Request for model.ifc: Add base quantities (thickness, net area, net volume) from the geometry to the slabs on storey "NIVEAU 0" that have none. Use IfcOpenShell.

First a look at what the model holds.

```python
import ifcopenshell
import ifcopenshell.util.element
import ifcopenshell.util.unit

model = ifcopenshell.open("model.ifc")
print(model.schema)
for unit_type in ("LENGTHUNIT", "AREAUNIT", "VOLUMEUNIT"):
    print(unit_type, ifcopenshell.util.unit.calculate_unit_scale(model, unit_type))
storey = next(s for s in model.by_type("IfcBuildingStorey") if s.Name == "NIVEAU 0")
slabs = [e for e in ifcopenshell.util.element.get_decomposition(storey) if e.is_a("IfcSlab")]
for e in sorted(slabs, key=lambda e: e.id()):
    print(e.id(), e.is_a(), e.Name, list(ifcopenshell.util.element.get_psets(e, qtos_only=True)), sep=" | ")
```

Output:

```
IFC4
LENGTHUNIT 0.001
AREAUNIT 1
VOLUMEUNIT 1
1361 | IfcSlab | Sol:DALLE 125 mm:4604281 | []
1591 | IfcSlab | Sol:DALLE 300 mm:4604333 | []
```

```python
import ifcopenshell
import ifcopenshell.api.pset
import ifcopenshell.geom
import ifcopenshell.util.element
import ifcopenshell.util.shape
import ifcopenshell.util.unit

model = ifcopenshell.open("model.ifc")
unit_scale = ifcopenshell.util.unit.calculate_unit_scale(model)
area_scale = ifcopenshell.util.unit.calculate_unit_scale(model, "AREAUNIT")
volume_scale = ifcopenshell.util.unit.calculate_unit_scale(model, "VOLUMEUNIT")
settings = ifcopenshell.geom.settings()

storey = next(s for s in model.by_type("IfcBuildingStorey") if s.Name == "NIVEAU 0")
slabs = [e for e in ifcopenshell.util.element.get_decomposition(storey) if e.is_a("IfcSlab")]

for e in sorted(slabs, key=lambda e: e.id()):
    if ifcopenshell.util.element.get_psets(e, qtos_only=True, should_inherit=False):
        continue
    # Geometry comes back in metres, in the element's own axes.
    shape = ifcopenshell.geom.create_shape(settings, e)
    values = {
        "Width": ifcopenshell.util.shape.get_z(shape.geometry) / unit_scale,
        "NetArea": ifcopenshell.util.shape.get_footprint_area(shape.geometry) / area_scale,
        "NetVolume": ifcopenshell.util.shape.get_volume(shape.geometry) / volume_scale,
    }
    qto = ifcopenshell.api.pset.add_qto(model, product=e, name="Qto_SlabBaseQuantities")
    ifcopenshell.api.pset.edit_qto(model, qto=qto, properties=values)
    print(e.id(), {k: round(v, 3) for k, v in values.items()})

model.write("model_updated.ifc")
```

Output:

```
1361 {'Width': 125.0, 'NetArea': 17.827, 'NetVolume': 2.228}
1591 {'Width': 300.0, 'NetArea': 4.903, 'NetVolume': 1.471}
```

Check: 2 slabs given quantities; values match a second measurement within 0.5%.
